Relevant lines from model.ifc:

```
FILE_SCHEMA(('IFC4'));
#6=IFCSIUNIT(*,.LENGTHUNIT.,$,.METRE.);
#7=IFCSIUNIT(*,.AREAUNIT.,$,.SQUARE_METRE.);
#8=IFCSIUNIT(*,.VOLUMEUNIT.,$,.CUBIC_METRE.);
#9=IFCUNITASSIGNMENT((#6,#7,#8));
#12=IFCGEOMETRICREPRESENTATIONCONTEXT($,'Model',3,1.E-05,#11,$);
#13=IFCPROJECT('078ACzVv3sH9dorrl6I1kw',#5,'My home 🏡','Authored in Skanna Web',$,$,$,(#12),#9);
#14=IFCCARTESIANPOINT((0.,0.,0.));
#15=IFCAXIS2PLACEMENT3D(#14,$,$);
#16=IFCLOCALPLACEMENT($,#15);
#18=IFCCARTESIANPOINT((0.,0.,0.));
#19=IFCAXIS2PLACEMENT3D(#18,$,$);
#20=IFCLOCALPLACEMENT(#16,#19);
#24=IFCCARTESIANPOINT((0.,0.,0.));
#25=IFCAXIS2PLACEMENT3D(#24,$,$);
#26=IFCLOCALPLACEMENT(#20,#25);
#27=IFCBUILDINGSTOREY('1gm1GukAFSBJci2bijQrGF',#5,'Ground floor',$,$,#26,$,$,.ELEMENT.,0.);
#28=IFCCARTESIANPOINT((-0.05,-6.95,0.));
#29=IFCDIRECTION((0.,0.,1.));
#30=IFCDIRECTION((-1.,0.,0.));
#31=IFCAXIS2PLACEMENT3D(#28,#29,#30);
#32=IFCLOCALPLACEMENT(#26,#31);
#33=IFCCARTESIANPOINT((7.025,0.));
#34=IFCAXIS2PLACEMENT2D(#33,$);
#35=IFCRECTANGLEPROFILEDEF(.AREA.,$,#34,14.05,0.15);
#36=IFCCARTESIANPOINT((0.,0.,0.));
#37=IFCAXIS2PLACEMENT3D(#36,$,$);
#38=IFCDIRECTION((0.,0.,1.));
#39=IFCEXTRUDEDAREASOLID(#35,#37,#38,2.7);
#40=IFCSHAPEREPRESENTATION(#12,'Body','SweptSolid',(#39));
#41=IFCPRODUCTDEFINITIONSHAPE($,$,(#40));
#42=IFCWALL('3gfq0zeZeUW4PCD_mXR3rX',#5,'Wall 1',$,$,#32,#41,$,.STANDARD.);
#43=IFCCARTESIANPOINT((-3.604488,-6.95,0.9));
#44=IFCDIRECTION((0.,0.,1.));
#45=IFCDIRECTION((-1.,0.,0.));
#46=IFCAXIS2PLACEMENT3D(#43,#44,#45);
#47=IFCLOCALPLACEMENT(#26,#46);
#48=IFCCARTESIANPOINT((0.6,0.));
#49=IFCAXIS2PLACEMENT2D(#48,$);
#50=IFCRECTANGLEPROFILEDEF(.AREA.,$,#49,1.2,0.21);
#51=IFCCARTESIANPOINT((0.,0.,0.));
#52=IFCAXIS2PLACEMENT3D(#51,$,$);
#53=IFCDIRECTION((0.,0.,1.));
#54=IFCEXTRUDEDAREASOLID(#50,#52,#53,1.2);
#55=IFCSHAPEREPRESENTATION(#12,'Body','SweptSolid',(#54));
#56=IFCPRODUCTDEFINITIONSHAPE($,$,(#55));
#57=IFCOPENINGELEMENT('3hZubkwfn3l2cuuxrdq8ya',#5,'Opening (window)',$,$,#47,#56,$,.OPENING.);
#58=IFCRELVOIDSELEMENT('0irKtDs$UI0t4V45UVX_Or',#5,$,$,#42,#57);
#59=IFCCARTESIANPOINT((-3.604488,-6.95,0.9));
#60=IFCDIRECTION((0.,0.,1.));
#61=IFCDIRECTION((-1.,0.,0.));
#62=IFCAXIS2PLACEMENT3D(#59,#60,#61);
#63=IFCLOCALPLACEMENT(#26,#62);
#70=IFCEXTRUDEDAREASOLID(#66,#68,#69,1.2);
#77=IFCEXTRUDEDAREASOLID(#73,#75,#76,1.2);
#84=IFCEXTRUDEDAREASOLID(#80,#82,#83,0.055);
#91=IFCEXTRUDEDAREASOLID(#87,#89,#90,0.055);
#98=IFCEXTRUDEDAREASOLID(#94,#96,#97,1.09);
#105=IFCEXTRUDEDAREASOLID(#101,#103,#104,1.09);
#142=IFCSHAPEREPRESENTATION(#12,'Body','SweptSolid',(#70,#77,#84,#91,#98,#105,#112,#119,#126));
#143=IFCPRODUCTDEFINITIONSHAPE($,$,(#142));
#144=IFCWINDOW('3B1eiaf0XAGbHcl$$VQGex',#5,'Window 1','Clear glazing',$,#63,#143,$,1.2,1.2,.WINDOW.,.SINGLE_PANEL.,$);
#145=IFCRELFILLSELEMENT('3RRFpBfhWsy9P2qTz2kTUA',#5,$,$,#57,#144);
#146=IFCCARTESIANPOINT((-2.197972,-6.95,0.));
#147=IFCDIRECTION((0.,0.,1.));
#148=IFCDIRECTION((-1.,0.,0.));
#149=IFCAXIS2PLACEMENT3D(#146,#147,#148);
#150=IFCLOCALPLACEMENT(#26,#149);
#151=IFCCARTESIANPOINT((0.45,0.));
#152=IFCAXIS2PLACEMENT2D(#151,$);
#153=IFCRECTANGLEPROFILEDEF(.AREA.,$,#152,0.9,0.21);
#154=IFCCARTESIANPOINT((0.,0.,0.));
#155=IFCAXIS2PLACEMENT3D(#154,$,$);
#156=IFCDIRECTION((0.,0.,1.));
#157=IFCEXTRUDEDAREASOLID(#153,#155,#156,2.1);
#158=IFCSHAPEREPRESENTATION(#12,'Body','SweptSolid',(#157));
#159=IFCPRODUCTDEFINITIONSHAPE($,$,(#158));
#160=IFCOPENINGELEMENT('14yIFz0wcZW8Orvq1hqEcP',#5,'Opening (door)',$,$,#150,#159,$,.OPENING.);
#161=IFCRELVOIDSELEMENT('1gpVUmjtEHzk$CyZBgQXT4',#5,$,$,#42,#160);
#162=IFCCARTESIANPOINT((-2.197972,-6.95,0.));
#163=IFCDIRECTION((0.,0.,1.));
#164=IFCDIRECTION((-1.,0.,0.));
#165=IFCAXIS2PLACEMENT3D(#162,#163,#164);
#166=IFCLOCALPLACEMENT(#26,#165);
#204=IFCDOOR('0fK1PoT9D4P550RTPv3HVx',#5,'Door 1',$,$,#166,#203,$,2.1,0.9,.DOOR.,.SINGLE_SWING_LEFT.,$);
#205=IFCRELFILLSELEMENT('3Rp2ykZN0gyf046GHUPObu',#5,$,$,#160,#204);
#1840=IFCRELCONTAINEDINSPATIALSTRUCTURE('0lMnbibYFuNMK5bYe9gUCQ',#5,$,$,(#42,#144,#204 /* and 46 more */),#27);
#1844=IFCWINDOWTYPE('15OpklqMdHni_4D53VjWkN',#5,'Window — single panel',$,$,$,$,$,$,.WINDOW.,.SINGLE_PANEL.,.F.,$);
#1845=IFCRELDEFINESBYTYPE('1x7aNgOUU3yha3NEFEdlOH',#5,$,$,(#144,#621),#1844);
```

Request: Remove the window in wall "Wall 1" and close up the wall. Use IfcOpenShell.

```python
import ifcopenshell
import ifcopenshell.api.feature
import ifcopenshell.api.root
import ifcopenshell.geom
import ifcopenshell.util.shape

model = ifcopenshell.open("model.ifc")
settings = ifcopenshell.geom.settings()


def volume(element):
    """Net volume in cubic metres, openings subtracted."""
    shape = ifcopenshell.geom.create_shape(settings, element)
    return ifcopenshell.util.shape.get_volume(shape.geometry)


window = model.by_guid("3B1eiaf0XAGbHcl$$VQGex")
opening = window.FillsVoids[0].RelatingOpeningElement
wall = opening.VoidsElements[0].RelatingBuildingElement
before = volume(wall)

ifcopenshell.api.root.remove_product(model, product=window)
ifcopenshell.api.feature.remove_feature(model, feature=opening)

after = volume(wall)

print(f"wall volume {before:.3f} -> {after:.3f} m3")

model.write("model_updated.ifc")
```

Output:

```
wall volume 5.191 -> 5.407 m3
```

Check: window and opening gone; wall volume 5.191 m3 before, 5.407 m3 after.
